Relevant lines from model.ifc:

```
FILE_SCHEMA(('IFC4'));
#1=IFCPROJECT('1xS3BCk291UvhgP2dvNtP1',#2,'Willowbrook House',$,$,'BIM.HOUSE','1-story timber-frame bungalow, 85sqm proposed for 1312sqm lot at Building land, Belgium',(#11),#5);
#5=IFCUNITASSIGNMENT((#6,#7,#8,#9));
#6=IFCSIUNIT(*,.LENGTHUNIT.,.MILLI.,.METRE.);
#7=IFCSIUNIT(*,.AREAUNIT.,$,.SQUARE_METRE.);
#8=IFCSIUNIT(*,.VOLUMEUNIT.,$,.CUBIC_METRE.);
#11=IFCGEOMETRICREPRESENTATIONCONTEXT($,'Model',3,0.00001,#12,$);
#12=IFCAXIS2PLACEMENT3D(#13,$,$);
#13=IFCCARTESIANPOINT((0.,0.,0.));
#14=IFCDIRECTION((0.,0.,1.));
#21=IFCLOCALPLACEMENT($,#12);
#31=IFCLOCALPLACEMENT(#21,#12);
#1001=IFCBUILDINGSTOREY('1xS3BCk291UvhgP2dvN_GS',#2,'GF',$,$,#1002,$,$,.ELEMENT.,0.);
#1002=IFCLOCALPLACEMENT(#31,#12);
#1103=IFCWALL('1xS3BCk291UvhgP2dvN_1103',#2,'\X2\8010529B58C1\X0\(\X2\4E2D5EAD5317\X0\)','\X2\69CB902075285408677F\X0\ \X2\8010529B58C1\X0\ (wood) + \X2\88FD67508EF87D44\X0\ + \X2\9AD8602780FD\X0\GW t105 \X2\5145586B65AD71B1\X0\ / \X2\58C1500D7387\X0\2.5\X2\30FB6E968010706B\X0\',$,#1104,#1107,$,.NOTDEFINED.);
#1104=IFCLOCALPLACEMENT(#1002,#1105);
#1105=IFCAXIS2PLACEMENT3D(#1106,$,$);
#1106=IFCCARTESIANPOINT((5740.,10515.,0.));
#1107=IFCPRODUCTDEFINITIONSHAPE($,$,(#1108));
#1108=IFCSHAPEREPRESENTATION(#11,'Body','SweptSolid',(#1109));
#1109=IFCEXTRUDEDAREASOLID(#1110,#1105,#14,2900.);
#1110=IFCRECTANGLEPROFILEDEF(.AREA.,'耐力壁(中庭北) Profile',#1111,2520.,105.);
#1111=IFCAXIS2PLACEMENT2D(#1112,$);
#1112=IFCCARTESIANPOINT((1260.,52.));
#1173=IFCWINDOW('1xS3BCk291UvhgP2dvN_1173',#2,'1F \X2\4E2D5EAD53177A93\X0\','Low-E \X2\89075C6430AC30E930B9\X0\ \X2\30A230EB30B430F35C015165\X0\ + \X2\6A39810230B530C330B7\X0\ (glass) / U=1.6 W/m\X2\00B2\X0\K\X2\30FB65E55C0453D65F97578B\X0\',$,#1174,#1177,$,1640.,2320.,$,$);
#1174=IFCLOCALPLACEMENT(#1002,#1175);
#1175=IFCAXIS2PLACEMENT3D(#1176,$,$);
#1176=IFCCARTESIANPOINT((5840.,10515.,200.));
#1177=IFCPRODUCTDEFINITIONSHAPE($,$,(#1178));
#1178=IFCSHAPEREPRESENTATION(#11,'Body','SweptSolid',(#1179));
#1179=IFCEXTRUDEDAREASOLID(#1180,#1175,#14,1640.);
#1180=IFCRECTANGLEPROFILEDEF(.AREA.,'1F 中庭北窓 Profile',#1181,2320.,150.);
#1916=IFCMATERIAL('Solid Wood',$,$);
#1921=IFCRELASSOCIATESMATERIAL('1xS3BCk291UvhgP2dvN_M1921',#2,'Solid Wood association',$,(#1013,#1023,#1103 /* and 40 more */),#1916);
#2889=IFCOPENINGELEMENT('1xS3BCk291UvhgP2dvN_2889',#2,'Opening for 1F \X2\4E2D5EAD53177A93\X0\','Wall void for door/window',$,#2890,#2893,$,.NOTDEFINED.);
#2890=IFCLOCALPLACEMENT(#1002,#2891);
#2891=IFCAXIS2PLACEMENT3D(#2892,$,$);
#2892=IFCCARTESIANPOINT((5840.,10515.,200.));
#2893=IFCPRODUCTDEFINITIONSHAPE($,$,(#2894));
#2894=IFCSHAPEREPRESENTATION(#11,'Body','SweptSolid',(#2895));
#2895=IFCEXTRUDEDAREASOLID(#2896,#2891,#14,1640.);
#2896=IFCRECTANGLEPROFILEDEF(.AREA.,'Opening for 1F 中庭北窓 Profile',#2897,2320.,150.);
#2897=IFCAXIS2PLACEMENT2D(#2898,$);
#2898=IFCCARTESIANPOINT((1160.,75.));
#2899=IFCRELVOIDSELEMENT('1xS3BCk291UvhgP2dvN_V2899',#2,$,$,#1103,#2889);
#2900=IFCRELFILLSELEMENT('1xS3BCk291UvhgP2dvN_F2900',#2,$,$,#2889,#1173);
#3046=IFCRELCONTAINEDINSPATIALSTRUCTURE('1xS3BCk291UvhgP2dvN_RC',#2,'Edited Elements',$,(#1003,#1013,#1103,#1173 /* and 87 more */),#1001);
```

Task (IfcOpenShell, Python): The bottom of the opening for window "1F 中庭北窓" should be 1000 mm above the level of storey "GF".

```python
import numpy as np
import ifcopenshell
import ifcopenshell.api.geometry
import ifcopenshell.geom
import ifcopenshell.util.element
import ifcopenshell.util.placement
import ifcopenshell.util.shape
import ifcopenshell.util.unit

model = ifcopenshell.open("model.ifc")
unit_scale = ifcopenshell.util.unit.calculate_unit_scale(model)

window = model.by_guid("1xS3BCk291UvhgP2dvN_1173")
opening = window.FillsVoids[0].RelatingOpeningElement
storey = ifcopenshell.util.element.get_container(window, ifc_class="IfcBuildingStorey")
level = ifcopenshell.util.placement.get_local_placement(storey.ObjectPlacement)[2, 3]

# The opening's origin need not be at the sill, so measure its lowest point.
shape = ifcopenshell.geom.create_shape(ifcopenshell.geom.settings(), opening)
bottom = ifcopenshell.util.shape.get_shape_bottom_elevation(shape, shape.geometry) / unit_scale
dz = level + 1 / unit_scale - bottom

shift = np.array([0.0, 0.0, dz])
# The window is not placed relative to its opening, so move both.
for product in (opening, window):
    matrix = ifcopenshell.util.placement.get_local_placement(product.ObjectPlacement)
    matrix[:3, 3] += shift
    ifcopenshell.api.geometry.edit_object_placement(model, product=product, matrix=matrix, is_si=False)

print(f"moved by {dz * unit_scale:+.3f} m")

model.write("model_updated.ifc")
```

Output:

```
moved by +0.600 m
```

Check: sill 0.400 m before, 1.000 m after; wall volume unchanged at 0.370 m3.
